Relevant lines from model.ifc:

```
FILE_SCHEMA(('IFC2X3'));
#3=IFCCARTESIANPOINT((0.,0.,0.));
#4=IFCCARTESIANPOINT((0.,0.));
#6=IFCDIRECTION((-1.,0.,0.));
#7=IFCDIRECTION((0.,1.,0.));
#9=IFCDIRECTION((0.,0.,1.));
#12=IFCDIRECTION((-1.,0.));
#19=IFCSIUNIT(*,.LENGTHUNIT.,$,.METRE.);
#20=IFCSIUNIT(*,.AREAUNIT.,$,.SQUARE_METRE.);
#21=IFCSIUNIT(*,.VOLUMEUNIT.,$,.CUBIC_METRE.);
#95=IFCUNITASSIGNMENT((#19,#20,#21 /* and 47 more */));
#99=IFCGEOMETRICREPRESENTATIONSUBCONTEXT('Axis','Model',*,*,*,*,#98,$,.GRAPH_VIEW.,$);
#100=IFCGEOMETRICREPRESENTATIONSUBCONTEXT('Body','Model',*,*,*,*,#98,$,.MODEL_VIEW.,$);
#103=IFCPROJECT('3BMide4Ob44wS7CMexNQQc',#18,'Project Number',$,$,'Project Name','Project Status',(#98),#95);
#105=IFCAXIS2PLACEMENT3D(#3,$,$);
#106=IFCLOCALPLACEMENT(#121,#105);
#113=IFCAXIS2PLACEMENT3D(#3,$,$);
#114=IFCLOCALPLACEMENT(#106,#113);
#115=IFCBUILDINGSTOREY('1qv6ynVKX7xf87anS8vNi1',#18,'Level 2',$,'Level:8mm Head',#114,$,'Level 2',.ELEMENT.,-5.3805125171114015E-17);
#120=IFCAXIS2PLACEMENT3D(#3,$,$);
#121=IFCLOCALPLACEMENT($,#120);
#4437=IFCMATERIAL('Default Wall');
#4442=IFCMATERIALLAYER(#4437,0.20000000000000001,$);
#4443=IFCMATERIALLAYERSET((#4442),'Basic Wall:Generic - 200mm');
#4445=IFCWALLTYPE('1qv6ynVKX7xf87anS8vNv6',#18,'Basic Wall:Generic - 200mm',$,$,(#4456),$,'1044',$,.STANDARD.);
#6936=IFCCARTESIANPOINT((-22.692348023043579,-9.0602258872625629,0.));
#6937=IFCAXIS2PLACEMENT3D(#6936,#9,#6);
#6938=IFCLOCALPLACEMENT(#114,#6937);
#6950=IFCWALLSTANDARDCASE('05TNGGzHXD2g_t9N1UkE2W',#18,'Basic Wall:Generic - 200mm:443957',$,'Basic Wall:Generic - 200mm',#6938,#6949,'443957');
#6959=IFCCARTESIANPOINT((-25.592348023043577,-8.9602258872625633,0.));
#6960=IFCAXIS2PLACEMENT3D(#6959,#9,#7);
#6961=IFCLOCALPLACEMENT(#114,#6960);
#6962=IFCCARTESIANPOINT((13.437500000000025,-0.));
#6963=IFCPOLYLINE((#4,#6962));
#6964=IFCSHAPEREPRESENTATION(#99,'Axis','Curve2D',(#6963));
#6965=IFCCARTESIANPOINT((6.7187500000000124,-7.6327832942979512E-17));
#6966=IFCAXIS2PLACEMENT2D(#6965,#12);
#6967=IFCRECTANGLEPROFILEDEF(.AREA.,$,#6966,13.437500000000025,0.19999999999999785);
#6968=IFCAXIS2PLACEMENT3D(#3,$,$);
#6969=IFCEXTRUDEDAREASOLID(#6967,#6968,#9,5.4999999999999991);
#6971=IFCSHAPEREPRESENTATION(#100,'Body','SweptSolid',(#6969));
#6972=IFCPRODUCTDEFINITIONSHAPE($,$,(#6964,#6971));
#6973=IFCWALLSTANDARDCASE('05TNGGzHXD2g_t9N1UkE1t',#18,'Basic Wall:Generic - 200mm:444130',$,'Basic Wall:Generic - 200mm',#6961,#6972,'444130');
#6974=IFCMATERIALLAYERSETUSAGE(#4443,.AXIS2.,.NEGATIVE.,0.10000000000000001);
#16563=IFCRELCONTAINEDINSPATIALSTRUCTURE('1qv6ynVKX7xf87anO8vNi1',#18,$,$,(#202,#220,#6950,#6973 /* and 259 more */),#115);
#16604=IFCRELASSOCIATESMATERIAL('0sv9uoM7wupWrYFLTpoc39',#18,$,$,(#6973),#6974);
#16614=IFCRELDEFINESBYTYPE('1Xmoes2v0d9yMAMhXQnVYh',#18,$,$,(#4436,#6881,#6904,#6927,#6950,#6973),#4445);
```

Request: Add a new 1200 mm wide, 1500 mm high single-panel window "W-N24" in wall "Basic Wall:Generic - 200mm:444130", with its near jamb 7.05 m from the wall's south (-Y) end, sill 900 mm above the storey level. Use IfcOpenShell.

```python
import numpy as np
import ifcopenshell
import ifcopenshell.api.feature
import ifcopenshell.api.geometry
import ifcopenshell.api.root
import ifcopenshell.api.spatial
import ifcopenshell.api.type
import ifcopenshell.geom
import ifcopenshell.util.element
import ifcopenshell.util.placement
import ifcopenshell.util.representation
import ifcopenshell.util.shape
import ifcopenshell.util.unit

model = ifcopenshell.open("model.ifc")
unit_scale = ifcopenshell.util.unit.calculate_unit_scale(model)
settings = ifcopenshell.geom.settings()


def volume(element):
    """Net volume in cubic metres, openings subtracted."""
    shape = ifcopenshell.geom.create_shape(settings, element)
    return ifcopenshell.util.shape.get_volume(shape.geometry)


wall = model.by_guid("05TNGGzHXD2g_t9N1UkE1t")
storey = ifcopenshell.util.element.get_container(wall, ifc_class="IfcBuildingStorey")
context = ifcopenshell.util.representation.get_context(model, "Model", "Body", "MODEL_VIEW")
before = volume(wall)

width, height, from_end, sill = 1.2, 1.5, 7.05, 0.9  # metres

# The wall runs along its own X axis, and the end named is its -X end.
wall_shape = ifcopenshell.geom.create_shape(settings, wall)
x, y, z = ifcopenshell.util.shape.get_vertices(wall_shape.geometry).T
start = x.min() + from_end
face, thickness = float(y.min()), float(y.max() - y.min())
wall_matrix = ifcopenshell.util.placement.get_local_placement(wall.ObjectPlacement)
level = ifcopenshell.util.placement.get_local_placement(storey.ObjectPlacement)[2, 3]


def in_wall(x, y):
    """Placement at x, y metres in the wall's axes, at sill height."""
    matrix = wall_matrix.copy()
    matrix[:, 3] = wall_matrix @ np.array([x / unit_scale, y / unit_scale, 0.0, 1.0])
    matrix[2, 3] = level + sill / unit_scale
    return matrix


# Opening: a box that overshoots both wall faces by 50 mm.
opening = ifcopenshell.api.root.create_entity(model, ifc_class="IfcOpeningElement")
box = ifcopenshell.api.geometry.add_wall_representation(
    model, context=context, length=width, height=height, thickness=thickness + 0.1
)
ifcopenshell.api.geometry.assign_representation(model, product=opening, representation=box)
ifcopenshell.api.geometry.edit_object_placement(model, product=opening, matrix=in_wall(start, face - 0.05), is_si=False)
ifcopenshell.api.feature.add_feature(model, feature=opening, element=wall)

window = ifcopenshell.api.root.create_entity(model, ifc_class="IfcWindow", name="W-N24")
window.OverallWidth, window.OverallHeight = width / unit_scale, height / unit_scale
body = ifcopenshell.api.geometry.add_window_representation(
    model,
    context=context,
    overall_width=window.OverallWidth,
    overall_height=window.OverallHeight,
    partition_type="SINGLE_PANEL",
)
ifcopenshell.api.geometry.assign_representation(model, product=window, representation=body)
ifcopenshell.api.spatial.assign_container(model, products=[window], relating_structure=storey)
fills = ifcopenshell.api.feature.add_filling(model, opening=opening, element=window)
fills.OwnerHistory = window.OwnerHistory  # required in IFC2X3

# IFC2X3 keeps the operation on the window style.
style = ifcopenshell.api.root.create_entity(model, ifc_class="IfcWindowStyle", name="W-N24")
style.OperationType, style.ConstructionType = "SINGLE_PANEL", "NOTDEFINED"
style.ParameterTakesPrecedence = style.Sizeable = False
ifcopenshell.api.type.assign_type(model, related_objects=[window], relating_type=style)

# Centre the window in the wall's thickness.
ifcopenshell.api.geometry.edit_object_placement(model, product=window, matrix=in_wall(start, face), is_si=False)
window_shape = ifcopenshell.geom.create_shape(settings, window)
depth = ifcopenshell.util.shape.get_vertices(window_shape.geometry)[:, 1]
offset = face + thickness / 2 - (depth.min() + depth.max()) / 2
ifcopenshell.api.geometry.edit_object_placement(model, product=window, matrix=in_wall(start, offset), is_si=False)

after = volume(wall)

print(f"wall volume {before:.3f} -> {after:.3f} m3")

model.write("model-out.ifc")
```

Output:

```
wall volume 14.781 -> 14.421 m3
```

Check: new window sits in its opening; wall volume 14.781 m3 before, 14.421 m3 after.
